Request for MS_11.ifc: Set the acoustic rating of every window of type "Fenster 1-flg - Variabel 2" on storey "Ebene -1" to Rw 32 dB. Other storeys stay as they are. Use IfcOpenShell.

First a look at what the model holds.

```python
import ifcopenshell
import ifcopenshell.util.element

model = ifcopenshell.open("MS_11.ifc")
print(model.schema)
storey = next(s for s in model.by_type("IfcBuildingStorey") if s.Name == "Ebene -1")
windows = [e for e in ifcopenshell.util.element.get_decomposition(storey) if e.is_a("IfcWindow")]
seen = {}
for e in windows:
    element_type = ifcopenshell.util.element.get_type(e)
    key = (element_type.Name if element_type != e and element_type else None, ifcopenshell.util.element.get_pset(e, "Pset_WindowCommon", "AcousticRating"))
    seen[key] = seen.get(key, 0) + 1
for (name, value), count in sorted(seen.items(), key=str):
    print(count, "x", name, "|", value)
```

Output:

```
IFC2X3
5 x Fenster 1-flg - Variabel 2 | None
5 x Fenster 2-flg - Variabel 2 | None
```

```python
import ifcopenshell
import ifcopenshell.api.pset
import ifcopenshell.util.element

model = ifcopenshell.open("MS_11.ifc")

storey = next(s for s in model.by_type("IfcBuildingStorey") if s.Name == "Ebene -1")
windows = [e for e in ifcopenshell.util.element.get_decomposition(storey) if e.is_a("IfcWindow")]

count = 0
for e in windows:
    element_type = ifcopenshell.util.element.get_type(e)
    if element_type in (None, e) or element_type.Name != "Fenster 1-flg - Variabel 2":
        continue
    # add_pset returns the element's existing set when there is one.
    pset = ifcopenshell.api.pset.add_pset(model, product=e, name="Pset_WindowCommon")
    ifcopenshell.api.pset.edit_pset(model, pset=pset, properties={"AcousticRating": "Rw 32 dB"})
    count += 1

print(count, "windows updated")

model.write("MS_11_rev.ifc")
```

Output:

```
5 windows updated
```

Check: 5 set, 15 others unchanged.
